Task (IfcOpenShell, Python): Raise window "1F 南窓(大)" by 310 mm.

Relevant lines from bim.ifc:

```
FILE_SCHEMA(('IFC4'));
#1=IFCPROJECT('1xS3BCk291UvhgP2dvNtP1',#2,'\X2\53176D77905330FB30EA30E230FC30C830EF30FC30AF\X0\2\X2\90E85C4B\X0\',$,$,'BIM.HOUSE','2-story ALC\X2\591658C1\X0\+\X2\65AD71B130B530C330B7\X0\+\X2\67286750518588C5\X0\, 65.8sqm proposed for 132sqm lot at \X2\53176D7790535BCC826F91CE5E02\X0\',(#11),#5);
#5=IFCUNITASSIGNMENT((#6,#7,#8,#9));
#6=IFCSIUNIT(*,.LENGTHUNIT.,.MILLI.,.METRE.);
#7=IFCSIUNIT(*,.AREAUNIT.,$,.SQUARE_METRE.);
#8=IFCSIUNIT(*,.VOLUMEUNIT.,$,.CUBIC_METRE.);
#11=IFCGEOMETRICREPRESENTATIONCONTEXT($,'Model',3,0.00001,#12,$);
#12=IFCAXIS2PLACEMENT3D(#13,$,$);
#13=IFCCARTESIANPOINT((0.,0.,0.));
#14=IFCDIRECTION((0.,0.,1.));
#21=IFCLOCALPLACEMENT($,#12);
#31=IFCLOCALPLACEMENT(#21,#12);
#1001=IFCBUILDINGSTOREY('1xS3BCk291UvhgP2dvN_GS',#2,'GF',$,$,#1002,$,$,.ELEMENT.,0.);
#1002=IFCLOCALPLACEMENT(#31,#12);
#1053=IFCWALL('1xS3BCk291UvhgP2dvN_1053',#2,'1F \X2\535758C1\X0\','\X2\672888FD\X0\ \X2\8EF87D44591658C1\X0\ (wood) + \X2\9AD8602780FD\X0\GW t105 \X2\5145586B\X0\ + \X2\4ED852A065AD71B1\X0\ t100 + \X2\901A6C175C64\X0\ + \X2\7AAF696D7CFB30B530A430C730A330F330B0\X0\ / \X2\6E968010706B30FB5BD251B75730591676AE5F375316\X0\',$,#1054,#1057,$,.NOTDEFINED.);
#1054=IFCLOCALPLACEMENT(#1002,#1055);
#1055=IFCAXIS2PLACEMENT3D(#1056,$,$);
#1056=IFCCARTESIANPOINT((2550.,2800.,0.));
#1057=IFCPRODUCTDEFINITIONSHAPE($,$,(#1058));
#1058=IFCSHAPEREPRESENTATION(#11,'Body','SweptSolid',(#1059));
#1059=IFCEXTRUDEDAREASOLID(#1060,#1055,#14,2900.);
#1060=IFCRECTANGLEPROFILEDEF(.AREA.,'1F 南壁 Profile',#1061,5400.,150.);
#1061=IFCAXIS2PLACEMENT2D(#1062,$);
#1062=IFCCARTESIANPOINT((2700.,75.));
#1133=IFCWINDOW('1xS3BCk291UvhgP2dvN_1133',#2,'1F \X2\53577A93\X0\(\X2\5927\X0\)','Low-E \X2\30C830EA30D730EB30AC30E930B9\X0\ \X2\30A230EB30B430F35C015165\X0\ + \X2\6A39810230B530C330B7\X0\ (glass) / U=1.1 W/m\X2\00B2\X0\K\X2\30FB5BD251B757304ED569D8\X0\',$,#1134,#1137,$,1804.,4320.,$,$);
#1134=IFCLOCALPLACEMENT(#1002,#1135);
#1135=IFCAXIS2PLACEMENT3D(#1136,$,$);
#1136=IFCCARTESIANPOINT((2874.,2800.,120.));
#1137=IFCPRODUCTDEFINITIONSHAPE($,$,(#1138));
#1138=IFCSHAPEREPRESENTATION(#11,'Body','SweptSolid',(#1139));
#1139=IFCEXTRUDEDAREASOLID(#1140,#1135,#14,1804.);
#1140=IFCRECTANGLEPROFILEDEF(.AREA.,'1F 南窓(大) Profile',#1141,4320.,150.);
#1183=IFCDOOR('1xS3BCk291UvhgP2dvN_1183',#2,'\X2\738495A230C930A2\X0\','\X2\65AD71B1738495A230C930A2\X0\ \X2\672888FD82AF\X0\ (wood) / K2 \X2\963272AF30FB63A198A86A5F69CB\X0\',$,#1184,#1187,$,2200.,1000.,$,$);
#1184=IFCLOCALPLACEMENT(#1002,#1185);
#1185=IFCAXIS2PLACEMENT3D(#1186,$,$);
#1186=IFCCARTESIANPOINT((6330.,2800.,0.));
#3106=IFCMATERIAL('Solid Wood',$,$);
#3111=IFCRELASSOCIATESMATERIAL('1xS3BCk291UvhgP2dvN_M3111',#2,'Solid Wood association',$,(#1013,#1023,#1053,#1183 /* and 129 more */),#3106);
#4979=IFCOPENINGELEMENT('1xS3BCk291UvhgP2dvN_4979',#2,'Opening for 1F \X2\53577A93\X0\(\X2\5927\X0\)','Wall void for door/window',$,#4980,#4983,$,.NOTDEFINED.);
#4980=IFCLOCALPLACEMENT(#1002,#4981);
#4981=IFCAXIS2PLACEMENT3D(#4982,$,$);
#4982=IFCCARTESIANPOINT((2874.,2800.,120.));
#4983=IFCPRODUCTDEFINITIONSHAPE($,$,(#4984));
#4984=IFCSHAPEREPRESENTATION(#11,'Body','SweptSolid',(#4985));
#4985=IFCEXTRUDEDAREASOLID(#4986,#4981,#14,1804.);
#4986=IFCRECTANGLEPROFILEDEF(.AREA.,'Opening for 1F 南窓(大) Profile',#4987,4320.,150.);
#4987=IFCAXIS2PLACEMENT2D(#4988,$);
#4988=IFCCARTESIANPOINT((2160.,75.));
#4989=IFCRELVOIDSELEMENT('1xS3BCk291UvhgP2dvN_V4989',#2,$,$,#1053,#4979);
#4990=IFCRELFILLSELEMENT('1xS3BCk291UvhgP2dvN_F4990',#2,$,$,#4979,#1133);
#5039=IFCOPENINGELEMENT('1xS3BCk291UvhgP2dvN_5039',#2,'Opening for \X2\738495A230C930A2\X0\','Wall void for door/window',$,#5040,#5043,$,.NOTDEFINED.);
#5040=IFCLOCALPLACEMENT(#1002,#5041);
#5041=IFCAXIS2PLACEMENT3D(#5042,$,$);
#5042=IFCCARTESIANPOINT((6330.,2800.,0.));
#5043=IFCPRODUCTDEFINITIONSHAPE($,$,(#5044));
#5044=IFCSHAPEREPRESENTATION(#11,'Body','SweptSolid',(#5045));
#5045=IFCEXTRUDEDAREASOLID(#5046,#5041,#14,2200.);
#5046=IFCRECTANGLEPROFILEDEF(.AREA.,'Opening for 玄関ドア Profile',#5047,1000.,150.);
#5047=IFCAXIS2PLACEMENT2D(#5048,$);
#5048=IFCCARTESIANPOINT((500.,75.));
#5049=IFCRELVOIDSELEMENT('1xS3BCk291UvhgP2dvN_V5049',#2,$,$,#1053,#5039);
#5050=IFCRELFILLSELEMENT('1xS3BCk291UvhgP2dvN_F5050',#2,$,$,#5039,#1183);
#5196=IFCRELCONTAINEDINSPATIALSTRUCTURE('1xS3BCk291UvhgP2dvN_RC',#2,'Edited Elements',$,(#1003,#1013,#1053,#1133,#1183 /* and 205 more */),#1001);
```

```python
import numpy as np
import ifcopenshell
import ifcopenshell.api.geometry
import ifcopenshell.util.placement
import ifcopenshell.util.unit

model = ifcopenshell.open("bim.ifc")
unit_scale = ifcopenshell.util.unit.calculate_unit_scale(model)

window = model.by_guid("1xS3BCk291UvhgP2dvN_1133")
opening = window.FillsVoids[0].RelatingOpeningElement
dz = 310.0

shift = np.array([0.0, 0.0, dz])
# The window is not placed relative to its opening, so move both.
for product in (opening, window):
    matrix = ifcopenshell.util.placement.get_local_placement(product.ObjectPlacement)
    matrix[:3, 3] += shift
    ifcopenshell.api.geometry.edit_object_placement(model, product=product, matrix=matrix, is_si=False)

print(f"moved by {dz * unit_scale:+.3f} m")

model.write("bim_edited.ifc")
```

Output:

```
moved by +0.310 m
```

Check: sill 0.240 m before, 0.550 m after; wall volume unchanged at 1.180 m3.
